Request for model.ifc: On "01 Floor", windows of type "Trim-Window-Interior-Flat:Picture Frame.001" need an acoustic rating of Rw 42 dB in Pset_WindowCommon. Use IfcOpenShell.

First a look at what the model holds.

```python
import ifcopenshell
import ifcopenshell.util.element

model = ifcopenshell.open("model.ifc")
print(model.schema)
storey = next(s for s in model.by_type("IfcBuildingStorey") if s.Name == "01 Floor")
windows = [e for e in ifcopenshell.util.element.get_decomposition(storey) if e.is_a("IfcWindow")]
seen = {}
for e in windows:
    element_type = ifcopenshell.util.element.get_type(e)
    key = (element_type.Name if element_type != e and element_type else None, ifcopenshell.util.element.get_pset(e, "Pset_WindowCommon", "AcousticRating"))
    seen[key] = seen.get(key, 0) + 1
for (name, value), count in sorted(seen.items(), key=str):
    print(count, "x", name, "|", value)
```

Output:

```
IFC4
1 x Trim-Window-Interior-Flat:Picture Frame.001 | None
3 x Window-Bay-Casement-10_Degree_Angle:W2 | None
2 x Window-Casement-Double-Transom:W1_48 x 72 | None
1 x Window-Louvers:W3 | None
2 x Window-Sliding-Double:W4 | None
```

```python
import ifcopenshell
import ifcopenshell.api.pset
import ifcopenshell.util.element

model = ifcopenshell.open("model.ifc")

storey = next(s for s in model.by_type("IfcBuildingStorey") if s.Name == "01 Floor")
windows = [e for e in ifcopenshell.util.element.get_decomposition(storey) if e.is_a("IfcWindow")]

count = 0
for e in windows:
    element_type = ifcopenshell.util.element.get_type(e)
    if element_type in (None, e) or element_type.Name != "Trim-Window-Interior-Flat:Picture Frame.001":
        continue
    # add_pset returns the element's existing set when there is one.
    pset = ifcopenshell.api.pset.add_pset(model, product=e, name="Pset_WindowCommon")
    ifcopenshell.api.pset.edit_pset(model, pset=pset, properties={"AcousticRating": "Rw 42 dB"})
    count += 1

print(count, "windows updated")

model.write("model_v2.ifc")
```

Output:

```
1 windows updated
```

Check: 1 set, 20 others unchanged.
